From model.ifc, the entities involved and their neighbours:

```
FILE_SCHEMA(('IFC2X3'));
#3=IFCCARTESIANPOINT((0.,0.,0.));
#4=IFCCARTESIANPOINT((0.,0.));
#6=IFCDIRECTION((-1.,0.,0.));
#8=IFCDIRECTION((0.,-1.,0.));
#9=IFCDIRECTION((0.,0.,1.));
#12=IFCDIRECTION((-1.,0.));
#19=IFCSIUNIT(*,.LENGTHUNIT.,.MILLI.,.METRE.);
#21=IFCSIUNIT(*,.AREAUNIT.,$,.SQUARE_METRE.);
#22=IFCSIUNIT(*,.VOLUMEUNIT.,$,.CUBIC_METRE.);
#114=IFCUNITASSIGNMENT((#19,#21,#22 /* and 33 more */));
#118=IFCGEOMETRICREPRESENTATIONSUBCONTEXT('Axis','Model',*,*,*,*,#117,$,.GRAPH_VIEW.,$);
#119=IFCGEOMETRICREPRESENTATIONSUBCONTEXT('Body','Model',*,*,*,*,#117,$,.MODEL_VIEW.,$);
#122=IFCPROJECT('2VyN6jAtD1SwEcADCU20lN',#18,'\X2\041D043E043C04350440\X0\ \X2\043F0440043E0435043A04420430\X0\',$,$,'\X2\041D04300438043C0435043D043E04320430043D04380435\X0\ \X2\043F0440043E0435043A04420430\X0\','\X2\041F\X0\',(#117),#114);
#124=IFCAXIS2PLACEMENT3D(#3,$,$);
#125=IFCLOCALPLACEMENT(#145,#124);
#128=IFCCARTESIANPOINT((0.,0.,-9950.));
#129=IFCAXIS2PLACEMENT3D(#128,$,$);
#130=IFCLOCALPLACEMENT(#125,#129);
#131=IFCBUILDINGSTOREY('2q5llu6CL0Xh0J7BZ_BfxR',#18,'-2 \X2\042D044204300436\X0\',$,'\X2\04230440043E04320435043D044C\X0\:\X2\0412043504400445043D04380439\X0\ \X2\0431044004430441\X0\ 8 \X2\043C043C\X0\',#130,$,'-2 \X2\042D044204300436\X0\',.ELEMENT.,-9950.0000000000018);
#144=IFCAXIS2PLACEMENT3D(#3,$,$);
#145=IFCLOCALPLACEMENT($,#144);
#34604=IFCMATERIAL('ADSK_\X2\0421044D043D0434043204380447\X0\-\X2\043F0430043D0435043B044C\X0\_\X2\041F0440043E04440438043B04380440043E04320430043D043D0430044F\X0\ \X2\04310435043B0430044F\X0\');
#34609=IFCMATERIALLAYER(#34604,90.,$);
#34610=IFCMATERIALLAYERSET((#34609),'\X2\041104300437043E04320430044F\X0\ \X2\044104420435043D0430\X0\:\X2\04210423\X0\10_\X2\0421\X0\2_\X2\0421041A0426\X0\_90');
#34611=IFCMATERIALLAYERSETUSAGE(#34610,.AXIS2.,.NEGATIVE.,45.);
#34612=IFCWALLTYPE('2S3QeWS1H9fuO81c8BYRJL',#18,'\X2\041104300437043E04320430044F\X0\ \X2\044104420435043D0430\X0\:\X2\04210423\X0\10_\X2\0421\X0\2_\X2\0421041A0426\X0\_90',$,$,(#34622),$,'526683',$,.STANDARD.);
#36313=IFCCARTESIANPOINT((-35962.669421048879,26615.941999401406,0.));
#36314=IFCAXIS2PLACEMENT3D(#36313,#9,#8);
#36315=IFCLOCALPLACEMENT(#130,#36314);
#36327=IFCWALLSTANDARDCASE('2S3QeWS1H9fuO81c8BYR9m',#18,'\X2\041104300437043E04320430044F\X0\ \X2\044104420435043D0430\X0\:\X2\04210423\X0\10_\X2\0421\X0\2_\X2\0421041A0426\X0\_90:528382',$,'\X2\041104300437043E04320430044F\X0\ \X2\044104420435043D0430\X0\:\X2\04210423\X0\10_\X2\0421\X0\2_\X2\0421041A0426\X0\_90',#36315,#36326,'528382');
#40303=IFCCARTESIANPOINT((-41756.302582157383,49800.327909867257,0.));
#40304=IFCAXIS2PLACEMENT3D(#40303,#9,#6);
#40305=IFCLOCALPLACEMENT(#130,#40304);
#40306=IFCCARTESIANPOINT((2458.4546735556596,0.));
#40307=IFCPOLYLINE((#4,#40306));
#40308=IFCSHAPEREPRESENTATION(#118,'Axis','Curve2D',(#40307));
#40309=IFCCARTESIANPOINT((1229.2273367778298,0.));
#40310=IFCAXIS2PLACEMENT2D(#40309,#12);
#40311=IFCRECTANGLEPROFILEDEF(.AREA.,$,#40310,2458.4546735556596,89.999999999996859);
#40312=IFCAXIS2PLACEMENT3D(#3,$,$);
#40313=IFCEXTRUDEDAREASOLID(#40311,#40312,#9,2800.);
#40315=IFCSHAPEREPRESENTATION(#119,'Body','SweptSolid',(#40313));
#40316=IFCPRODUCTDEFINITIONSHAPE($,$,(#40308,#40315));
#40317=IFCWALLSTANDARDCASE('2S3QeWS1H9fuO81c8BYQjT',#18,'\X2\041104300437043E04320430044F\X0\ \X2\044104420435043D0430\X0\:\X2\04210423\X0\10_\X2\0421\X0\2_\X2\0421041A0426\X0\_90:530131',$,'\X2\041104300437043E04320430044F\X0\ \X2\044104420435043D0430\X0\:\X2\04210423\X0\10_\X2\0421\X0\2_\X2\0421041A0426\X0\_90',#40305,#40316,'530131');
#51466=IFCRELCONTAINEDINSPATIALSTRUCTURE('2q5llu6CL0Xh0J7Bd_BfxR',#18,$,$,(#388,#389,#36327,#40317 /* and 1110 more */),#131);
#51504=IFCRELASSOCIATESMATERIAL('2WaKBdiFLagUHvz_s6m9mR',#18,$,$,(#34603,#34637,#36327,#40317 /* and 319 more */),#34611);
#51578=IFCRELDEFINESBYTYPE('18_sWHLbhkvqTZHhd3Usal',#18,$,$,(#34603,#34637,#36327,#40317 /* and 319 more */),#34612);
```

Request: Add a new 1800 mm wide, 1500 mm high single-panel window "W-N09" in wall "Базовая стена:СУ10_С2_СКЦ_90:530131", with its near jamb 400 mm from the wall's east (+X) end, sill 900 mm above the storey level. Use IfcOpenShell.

```python
import numpy as np
import ifcopenshell
import ifcopenshell.api.feature
import ifcopenshell.api.geometry
import ifcopenshell.api.root
import ifcopenshell.api.spatial
import ifcopenshell.api.type
import ifcopenshell.geom
import ifcopenshell.util.element
import ifcopenshell.util.placement
import ifcopenshell.util.representation
import ifcopenshell.util.shape
import ifcopenshell.util.unit

model = ifcopenshell.open("model.ifc")
unit_scale = ifcopenshell.util.unit.calculate_unit_scale(model)
settings = ifcopenshell.geom.settings()


def volume(element):
    """Net volume in cubic metres, openings subtracted."""
    shape = ifcopenshell.geom.create_shape(settings, element)
    return ifcopenshell.util.shape.get_volume(shape.geometry)


wall = model.by_id(40317)
storey = ifcopenshell.util.element.get_container(wall, ifc_class="IfcBuildingStorey")
context = ifcopenshell.util.representation.get_context(model, "Model", "Body", "MODEL_VIEW")
before = volume(wall)

width, height, from_end, sill = 1.8, 1.5, 0.4, 0.9  # metres

# The wall runs along its own X axis, and the end named is its -X end.
wall_shape = ifcopenshell.geom.create_shape(settings, wall)
x, y, z = ifcopenshell.util.shape.get_vertices(wall_shape.geometry).T
start = x.min() + from_end
face, thickness = float(y.min()), float(y.max() - y.min())
wall_matrix = ifcopenshell.util.placement.get_local_placement(wall.ObjectPlacement)
level = ifcopenshell.util.placement.get_local_placement(storey.ObjectPlacement)[2, 3]


def in_wall(x, y):
    """Placement at x, y metres in the wall's axes, at sill height."""
    matrix = wall_matrix.copy()
    matrix[:, 3] = wall_matrix @ np.array([x / unit_scale, y / unit_scale, 0.0, 1.0])
    matrix[2, 3] = level + sill / unit_scale
    return matrix


# Opening: a box that overshoots both wall faces by 50 mm.
opening = ifcopenshell.api.root.create_entity(model, ifc_class="IfcOpeningElement")
box = ifcopenshell.api.geometry.add_wall_representation(
    model, context=context, length=width, height=height, thickness=thickness + 0.1
)
ifcopenshell.api.geometry.assign_representation(model, product=opening, representation=box)
ifcopenshell.api.geometry.edit_object_placement(model, product=opening, matrix=in_wall(start, face - 0.05), is_si=False)
ifcopenshell.api.feature.add_feature(model, feature=opening, element=wall)

window = ifcopenshell.api.root.create_entity(model, ifc_class="IfcWindow", name="W-N09")
window.OverallWidth, window.OverallHeight = width / unit_scale, height / unit_scale
body = ifcopenshell.api.geometry.add_window_representation(
    model,
    context=context,
    overall_width=window.OverallWidth,
    overall_height=window.OverallHeight,
    partition_type="SINGLE_PANEL",
)
ifcopenshell.api.geometry.assign_representation(model, product=window, representation=body)
ifcopenshell.api.spatial.assign_container(model, products=[window], relating_structure=storey)
fills = ifcopenshell.api.feature.add_filling(model, opening=opening, element=window)
fills.OwnerHistory = window.OwnerHistory  # required in IFC2X3

# IFC2X3 keeps the operation on the window style.
style = ifcopenshell.api.root.create_entity(model, ifc_class="IfcWindowStyle", name="W-N09")
style.OperationType, style.ConstructionType = "SINGLE_PANEL", "NOTDEFINED"
style.ParameterTakesPrecedence = style.Sizeable = False
ifcopenshell.api.type.assign_type(model, related_objects=[window], relating_type=style)

# Centre the window in the wall's thickness.
ifcopenshell.api.geometry.edit_object_placement(model, product=window, matrix=in_wall(start, face), is_si=False)
window_shape = ifcopenshell.geom.create_shape(settings, window)
depth = ifcopenshell.util.shape.get_vertices(window_shape.geometry)[:, 1]
offset = face + thickness / 2 - (depth.min() + depth.max()) / 2
ifcopenshell.api.geometry.edit_object_placement(model, product=window, matrix=in_wall(start, offset), is_si=False)

after = volume(wall)

print(f"wall volume {before:.3f} -> {after:.3f} m3")

model.write("model-out.ifc")
```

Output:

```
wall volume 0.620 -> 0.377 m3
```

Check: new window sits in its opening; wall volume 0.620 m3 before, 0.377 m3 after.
